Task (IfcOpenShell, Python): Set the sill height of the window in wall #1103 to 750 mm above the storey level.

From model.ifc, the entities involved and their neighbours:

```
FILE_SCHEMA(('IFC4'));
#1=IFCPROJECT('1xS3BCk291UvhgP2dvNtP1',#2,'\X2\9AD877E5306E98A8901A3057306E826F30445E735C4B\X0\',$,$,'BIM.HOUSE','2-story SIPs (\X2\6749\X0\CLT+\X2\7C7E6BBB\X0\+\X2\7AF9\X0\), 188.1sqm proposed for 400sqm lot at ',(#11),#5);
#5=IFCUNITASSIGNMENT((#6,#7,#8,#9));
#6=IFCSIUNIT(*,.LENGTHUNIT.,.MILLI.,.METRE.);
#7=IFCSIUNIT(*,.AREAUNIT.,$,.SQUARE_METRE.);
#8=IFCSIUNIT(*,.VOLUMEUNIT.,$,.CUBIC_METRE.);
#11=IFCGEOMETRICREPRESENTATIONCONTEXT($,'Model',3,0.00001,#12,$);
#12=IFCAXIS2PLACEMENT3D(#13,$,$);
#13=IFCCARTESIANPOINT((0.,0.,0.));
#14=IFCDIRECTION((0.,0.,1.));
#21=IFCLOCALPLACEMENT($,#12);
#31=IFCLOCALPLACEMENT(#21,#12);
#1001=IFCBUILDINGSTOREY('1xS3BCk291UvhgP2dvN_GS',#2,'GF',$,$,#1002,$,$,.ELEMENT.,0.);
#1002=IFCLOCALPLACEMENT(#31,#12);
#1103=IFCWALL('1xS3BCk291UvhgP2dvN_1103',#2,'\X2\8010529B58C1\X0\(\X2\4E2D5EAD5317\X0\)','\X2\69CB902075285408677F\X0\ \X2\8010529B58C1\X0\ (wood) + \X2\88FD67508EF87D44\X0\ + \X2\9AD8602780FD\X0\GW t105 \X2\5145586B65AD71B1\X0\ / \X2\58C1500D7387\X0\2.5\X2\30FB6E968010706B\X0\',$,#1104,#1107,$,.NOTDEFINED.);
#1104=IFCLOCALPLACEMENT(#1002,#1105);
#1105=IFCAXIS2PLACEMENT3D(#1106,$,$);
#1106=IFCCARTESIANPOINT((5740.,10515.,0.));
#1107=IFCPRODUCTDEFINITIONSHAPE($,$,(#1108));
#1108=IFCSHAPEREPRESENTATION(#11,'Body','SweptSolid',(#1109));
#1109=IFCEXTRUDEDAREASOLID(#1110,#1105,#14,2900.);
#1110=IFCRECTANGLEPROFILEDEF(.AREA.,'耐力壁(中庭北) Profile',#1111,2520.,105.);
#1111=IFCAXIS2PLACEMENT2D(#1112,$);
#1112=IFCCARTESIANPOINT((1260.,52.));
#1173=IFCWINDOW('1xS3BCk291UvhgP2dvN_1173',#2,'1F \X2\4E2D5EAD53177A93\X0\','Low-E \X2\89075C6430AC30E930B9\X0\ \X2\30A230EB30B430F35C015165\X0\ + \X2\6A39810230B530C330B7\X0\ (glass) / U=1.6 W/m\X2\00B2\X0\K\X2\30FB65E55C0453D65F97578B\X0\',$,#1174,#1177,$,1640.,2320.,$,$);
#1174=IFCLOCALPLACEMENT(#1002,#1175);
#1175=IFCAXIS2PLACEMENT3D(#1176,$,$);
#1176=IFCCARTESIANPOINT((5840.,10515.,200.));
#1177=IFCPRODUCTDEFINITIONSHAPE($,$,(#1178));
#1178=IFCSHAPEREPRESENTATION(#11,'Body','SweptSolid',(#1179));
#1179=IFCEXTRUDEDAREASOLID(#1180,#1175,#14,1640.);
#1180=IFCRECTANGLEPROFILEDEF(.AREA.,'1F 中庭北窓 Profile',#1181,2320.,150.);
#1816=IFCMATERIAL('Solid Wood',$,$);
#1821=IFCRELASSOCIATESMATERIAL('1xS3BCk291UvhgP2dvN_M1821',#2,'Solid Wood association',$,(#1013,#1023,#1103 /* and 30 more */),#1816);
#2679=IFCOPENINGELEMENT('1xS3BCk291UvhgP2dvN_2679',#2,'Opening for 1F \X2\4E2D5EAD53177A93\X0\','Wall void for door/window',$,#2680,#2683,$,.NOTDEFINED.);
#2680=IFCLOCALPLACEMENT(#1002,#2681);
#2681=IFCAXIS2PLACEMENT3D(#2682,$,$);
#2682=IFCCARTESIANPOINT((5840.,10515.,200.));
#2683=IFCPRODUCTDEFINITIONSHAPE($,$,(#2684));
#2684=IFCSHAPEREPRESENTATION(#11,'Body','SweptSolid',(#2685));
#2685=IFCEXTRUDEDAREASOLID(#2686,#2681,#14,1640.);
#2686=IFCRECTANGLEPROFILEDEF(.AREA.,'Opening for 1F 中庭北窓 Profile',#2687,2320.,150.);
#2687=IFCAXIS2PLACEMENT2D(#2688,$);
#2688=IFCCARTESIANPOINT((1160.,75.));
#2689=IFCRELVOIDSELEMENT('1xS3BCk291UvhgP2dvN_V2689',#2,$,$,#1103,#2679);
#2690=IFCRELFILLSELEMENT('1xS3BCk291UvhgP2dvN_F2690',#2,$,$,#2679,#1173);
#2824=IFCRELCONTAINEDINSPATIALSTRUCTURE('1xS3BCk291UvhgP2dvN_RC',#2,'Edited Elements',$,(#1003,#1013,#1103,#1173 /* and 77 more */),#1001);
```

```python
import numpy as np
import ifcopenshell
import ifcopenshell.api.geometry
import ifcopenshell.geom
import ifcopenshell.util.element
import ifcopenshell.util.placement
import ifcopenshell.util.shape
import ifcopenshell.util.unit

model = ifcopenshell.open("model.ifc")
unit_scale = ifcopenshell.util.unit.calculate_unit_scale(model)

window = model.by_guid("1xS3BCk291UvhgP2dvN_1173")
opening = window.FillsVoids[0].RelatingOpeningElement
storey = ifcopenshell.util.element.get_container(window, ifc_class="IfcBuildingStorey")
level = ifcopenshell.util.placement.get_local_placement(storey.ObjectPlacement)[2, 3]

# The opening's origin need not be at the sill, so measure its lowest point.
shape = ifcopenshell.geom.create_shape(ifcopenshell.geom.settings(), opening)
bottom = ifcopenshell.util.shape.get_shape_bottom_elevation(shape, shape.geometry) / unit_scale
dz = level + 0.75 / unit_scale - bottom

shift = np.array([0.0, 0.0, dz])
# The window is not placed relative to its opening, so move both.
for product in (opening, window):
    matrix = ifcopenshell.util.placement.get_local_placement(product.ObjectPlacement)
    matrix[:3, 3] += shift
    ifcopenshell.api.geometry.edit_object_placement(model, product=product, matrix=matrix, is_si=False)

print(f"moved by {dz * unit_scale:+.3f} m")

model.write("model_rev.ifc")
```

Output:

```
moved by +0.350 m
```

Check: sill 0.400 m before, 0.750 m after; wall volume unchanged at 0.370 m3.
